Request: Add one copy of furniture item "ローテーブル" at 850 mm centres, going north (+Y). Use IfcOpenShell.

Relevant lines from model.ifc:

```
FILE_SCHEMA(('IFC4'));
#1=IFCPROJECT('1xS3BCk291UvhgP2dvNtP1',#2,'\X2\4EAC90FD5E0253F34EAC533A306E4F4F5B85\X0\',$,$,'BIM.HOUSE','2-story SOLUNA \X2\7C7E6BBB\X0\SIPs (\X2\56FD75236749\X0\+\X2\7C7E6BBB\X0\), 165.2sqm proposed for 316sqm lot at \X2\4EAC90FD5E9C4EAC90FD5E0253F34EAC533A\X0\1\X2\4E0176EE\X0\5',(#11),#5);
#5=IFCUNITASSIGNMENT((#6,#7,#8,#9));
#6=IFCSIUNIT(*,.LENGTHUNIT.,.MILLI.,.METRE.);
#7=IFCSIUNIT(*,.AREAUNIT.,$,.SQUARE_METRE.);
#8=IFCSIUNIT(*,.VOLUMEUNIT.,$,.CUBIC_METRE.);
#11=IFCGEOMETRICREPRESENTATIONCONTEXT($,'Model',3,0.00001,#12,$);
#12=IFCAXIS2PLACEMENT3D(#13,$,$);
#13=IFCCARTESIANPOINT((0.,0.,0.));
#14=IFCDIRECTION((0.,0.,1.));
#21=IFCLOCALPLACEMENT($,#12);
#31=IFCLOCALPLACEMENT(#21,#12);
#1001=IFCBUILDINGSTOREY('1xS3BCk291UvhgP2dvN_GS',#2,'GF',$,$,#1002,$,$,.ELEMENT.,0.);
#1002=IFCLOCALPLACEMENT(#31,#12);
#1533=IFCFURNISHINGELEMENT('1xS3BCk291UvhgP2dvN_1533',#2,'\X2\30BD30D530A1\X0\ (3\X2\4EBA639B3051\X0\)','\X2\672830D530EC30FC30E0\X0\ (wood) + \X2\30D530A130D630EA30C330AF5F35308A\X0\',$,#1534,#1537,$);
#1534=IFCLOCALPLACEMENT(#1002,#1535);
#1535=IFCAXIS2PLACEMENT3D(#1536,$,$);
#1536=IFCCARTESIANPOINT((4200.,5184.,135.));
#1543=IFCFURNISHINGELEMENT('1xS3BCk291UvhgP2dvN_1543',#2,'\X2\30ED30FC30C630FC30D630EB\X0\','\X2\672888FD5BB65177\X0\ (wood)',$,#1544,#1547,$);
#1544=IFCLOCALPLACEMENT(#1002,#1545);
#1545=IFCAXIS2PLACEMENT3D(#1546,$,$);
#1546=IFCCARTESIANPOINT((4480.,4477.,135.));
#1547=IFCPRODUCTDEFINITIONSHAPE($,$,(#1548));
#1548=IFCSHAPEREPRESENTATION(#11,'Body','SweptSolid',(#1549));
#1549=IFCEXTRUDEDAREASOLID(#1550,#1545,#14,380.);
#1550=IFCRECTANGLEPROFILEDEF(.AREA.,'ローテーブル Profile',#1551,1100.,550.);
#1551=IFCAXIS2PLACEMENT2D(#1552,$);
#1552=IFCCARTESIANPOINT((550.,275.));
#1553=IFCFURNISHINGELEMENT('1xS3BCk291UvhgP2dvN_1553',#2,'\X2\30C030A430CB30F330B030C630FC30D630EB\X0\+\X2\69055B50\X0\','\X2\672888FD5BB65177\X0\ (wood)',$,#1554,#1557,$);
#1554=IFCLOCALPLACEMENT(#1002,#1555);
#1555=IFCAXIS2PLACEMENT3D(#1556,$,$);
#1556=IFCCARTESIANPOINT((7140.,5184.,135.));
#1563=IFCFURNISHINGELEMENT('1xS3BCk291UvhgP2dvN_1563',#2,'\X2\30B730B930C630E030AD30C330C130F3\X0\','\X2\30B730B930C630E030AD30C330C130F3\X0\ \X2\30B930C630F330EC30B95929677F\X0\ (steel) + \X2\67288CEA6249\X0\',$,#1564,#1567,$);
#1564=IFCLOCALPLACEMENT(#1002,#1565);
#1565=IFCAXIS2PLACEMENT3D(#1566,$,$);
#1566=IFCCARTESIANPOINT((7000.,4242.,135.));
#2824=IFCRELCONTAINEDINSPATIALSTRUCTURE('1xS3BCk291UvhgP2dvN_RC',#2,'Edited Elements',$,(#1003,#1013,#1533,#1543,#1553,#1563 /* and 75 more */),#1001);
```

```python
import numpy as np
import ifcopenshell
import ifcopenshell.api.geometry
import ifcopenshell.api.root
import ifcopenshell.util.element
import ifcopenshell.util.placement

model = ifcopenshell.open("model.ifc")


def reuse_history(source, copy):
    """copy_class also copies each property set's owner history, people and application; keep the originals."""
    for rel in copy.IsDefinedBy:
        if rel.is_a("IfcRelDefinesByProperties") and (history := rel.RelatingPropertyDefinition.OwnerHistory):
            rel.RelatingPropertyDefinition.OwnerHistory = source.OwnerHistory
            ifcopenshell.util.element.remove_deep2(model, history)


source = model.by_guid("1xS3BCk291UvhgP2dvN_1543")
base = ifcopenshell.util.placement.get_local_placement(source.ObjectPlacement)
step = np.array([0.0, 1.0, 0.0]) * 850.0

for i in range(1, 2):
    copy = ifcopenshell.api.root.copy_class(model, product=source)
    copy.Representation = ifcopenshell.util.element.copy_deep(
        model, source.Representation, exclude=["IfcGeometricRepresentationContext", "IfcRepresentationMap"]
    )
    reuse_history(source, copy)
    matrix = base.copy()
    matrix[:3, 3] += i * step
    print("added at", matrix[:3, 3].round(3) + 0.0)
    ifcopenshell.api.geometry.edit_object_placement(model, product=copy, matrix=matrix, is_si=False)

model.write("model_updated.ifc")
```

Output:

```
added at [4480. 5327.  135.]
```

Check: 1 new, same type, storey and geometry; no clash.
